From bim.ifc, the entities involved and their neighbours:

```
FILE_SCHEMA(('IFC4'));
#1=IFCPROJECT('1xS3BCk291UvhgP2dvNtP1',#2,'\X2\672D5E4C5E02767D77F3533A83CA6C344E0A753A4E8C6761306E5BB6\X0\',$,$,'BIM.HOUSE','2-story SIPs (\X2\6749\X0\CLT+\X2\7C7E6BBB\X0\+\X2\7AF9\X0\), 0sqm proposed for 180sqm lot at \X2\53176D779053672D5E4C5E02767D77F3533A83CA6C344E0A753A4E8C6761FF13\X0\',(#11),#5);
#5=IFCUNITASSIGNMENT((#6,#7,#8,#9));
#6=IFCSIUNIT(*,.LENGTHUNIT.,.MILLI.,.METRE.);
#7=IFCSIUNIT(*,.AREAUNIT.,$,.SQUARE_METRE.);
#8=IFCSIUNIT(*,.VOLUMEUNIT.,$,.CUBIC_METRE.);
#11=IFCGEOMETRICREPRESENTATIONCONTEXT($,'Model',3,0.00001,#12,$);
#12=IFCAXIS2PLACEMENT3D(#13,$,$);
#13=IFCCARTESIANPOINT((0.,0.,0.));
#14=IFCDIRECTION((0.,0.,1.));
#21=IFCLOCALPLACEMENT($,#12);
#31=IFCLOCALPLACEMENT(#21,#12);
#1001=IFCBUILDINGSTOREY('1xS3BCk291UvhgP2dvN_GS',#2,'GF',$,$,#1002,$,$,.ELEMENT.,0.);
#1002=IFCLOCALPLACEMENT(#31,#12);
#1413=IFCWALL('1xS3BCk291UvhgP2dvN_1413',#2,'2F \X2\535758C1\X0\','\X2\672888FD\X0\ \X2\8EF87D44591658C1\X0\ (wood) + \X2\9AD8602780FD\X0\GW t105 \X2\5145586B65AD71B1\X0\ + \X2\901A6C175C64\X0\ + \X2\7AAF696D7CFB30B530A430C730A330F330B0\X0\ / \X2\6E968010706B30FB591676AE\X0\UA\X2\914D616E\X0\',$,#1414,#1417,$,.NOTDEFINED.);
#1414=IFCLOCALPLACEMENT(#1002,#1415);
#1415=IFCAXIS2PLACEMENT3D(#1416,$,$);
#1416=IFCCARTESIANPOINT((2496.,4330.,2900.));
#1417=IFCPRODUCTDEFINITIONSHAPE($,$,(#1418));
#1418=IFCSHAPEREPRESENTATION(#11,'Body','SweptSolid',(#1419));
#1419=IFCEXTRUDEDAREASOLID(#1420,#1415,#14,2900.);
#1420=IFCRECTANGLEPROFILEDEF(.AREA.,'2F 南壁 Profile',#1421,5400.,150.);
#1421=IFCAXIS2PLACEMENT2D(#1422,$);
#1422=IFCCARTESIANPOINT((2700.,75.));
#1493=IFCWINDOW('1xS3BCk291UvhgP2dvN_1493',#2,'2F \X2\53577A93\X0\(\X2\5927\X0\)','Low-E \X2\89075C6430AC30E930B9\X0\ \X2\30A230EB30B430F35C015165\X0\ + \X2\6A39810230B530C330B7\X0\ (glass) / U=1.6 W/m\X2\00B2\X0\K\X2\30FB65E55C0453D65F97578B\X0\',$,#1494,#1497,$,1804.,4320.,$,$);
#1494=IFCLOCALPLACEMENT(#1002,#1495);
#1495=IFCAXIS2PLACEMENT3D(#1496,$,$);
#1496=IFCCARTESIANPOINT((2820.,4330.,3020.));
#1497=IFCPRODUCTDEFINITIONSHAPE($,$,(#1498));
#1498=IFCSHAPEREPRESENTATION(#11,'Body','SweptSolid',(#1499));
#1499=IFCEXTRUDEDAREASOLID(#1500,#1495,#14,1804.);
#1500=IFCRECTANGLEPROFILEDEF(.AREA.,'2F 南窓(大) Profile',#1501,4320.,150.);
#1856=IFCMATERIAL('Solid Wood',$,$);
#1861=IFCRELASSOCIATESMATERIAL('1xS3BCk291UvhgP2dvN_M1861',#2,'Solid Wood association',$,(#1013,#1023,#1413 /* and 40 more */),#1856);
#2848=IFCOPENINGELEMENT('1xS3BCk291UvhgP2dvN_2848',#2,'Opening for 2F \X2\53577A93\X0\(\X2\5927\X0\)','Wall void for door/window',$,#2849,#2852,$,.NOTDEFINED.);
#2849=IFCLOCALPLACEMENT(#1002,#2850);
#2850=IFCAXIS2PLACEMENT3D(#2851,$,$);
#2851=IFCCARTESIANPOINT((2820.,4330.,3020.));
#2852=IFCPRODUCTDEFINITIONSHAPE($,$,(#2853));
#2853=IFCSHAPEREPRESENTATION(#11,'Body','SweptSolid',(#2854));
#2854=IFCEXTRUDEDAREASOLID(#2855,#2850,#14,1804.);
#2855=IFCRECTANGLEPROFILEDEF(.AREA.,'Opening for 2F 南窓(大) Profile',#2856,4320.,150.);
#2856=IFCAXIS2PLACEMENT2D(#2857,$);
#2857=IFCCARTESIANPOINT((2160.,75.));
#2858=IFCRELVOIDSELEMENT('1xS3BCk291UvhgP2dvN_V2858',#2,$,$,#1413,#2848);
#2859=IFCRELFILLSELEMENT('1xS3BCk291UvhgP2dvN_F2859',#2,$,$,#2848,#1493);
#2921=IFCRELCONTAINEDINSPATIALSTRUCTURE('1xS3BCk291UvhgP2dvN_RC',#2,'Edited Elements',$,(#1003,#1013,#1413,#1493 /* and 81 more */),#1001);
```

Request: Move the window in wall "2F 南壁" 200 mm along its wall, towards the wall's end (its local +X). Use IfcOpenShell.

```python
import ifcopenshell
import ifcopenshell.api.geometry
import ifcopenshell.util.placement
import ifcopenshell.util.unit

model = ifcopenshell.open("bim.ifc")
unit_scale = ifcopenshell.util.unit.calculate_unit_scale(model)

window = model.by_guid("1xS3BCk291UvhgP2dvN_1493")
opening = window.FillsVoids[0].RelatingOpeningElement
wall = opening.VoidsElements[0].RelatingBuildingElement

wall_matrix = ifcopenshell.util.placement.get_local_placement(wall.ObjectPlacement)
shift = wall_matrix[:3, 0] * 0.2 / unit_scale
before = ifcopenshell.util.placement.get_local_placement(window.ObjectPlacement)[:3, 3].copy()

# The window is not placed relative to its opening, so move both.
for product in (opening, window):
    matrix = ifcopenshell.util.placement.get_local_placement(product.ObjectPlacement)
    matrix[:3, 3] += shift
    ifcopenshell.api.geometry.edit_object_placement(model, product=product, matrix=matrix, is_si=False)

after = ifcopenshell.util.placement.get_local_placement(window.ObjectPlacement)[:3, 3]
print("window moved by", (after - before).round(3) + 0.0)

model.write("bim_v2.ifc")
```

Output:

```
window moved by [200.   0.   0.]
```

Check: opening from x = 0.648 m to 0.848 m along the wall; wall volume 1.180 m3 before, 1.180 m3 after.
